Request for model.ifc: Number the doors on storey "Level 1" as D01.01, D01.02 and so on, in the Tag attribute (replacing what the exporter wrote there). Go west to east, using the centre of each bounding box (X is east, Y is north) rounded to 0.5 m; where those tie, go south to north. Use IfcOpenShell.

First a look at what the model holds.

```python
import ifcopenshell
import ifcopenshell.util.element
import ifcopenshell.util.placement

model = ifcopenshell.open("model.ifc")
print(model.schema)
storey = next(s for s in model.by_type("IfcBuildingStorey") if s.Name == "Level 1")
doors = [e for e in ifcopenshell.util.element.get_decomposition(storey) if e.is_a("IfcDoor")]
for e in sorted(doors, key=lambda e: e.id()):
    origin = ifcopenshell.util.placement.get_local_placement(e.ObjectPlacement)[:3, 3]
    print(e.id(), e.Tag, e.Name, origin.round(2) + 0.0, sep=" | ")
```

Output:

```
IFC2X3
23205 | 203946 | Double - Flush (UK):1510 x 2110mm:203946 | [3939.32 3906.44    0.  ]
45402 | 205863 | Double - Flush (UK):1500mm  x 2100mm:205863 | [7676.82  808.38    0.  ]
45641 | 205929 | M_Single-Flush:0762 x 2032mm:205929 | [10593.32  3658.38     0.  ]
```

```python
import ifcopenshell
import ifcopenshell.geom
import ifcopenshell.util.element
import ifcopenshell.util.shape

model = ifcopenshell.open("model.ifc")
settings = ifcopenshell.geom.settings()
settings.set("use-world-coords", True)


def centre(element):
    shape = ifcopenshell.geom.create_shape(settings, element)
    return ifcopenshell.util.shape.get_bbox_centroid(shape.geometry)


storey = next(s for s in model.by_type("IfcBuildingStorey") if s.Name == "Level 1")
doors = [e for e in ifcopenshell.util.element.get_decomposition(storey) if e.is_a("IfcDoor")]

# Insertion points can sit at a corner or the storey origin, so sort by the geometry (in metres).
centres = {e: centre(e) for e in doors}
doors.sort(key=lambda e: (round(centres[e][0] / 0.5), centres[e][1]))

for i, e in enumerate(doors, start=1):
    number = f"D01.{i:02d}"
    e.Tag = number
    print(e.id(), number)

model.write("model_rev.ifc")
```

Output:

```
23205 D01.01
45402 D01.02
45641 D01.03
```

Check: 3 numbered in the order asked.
